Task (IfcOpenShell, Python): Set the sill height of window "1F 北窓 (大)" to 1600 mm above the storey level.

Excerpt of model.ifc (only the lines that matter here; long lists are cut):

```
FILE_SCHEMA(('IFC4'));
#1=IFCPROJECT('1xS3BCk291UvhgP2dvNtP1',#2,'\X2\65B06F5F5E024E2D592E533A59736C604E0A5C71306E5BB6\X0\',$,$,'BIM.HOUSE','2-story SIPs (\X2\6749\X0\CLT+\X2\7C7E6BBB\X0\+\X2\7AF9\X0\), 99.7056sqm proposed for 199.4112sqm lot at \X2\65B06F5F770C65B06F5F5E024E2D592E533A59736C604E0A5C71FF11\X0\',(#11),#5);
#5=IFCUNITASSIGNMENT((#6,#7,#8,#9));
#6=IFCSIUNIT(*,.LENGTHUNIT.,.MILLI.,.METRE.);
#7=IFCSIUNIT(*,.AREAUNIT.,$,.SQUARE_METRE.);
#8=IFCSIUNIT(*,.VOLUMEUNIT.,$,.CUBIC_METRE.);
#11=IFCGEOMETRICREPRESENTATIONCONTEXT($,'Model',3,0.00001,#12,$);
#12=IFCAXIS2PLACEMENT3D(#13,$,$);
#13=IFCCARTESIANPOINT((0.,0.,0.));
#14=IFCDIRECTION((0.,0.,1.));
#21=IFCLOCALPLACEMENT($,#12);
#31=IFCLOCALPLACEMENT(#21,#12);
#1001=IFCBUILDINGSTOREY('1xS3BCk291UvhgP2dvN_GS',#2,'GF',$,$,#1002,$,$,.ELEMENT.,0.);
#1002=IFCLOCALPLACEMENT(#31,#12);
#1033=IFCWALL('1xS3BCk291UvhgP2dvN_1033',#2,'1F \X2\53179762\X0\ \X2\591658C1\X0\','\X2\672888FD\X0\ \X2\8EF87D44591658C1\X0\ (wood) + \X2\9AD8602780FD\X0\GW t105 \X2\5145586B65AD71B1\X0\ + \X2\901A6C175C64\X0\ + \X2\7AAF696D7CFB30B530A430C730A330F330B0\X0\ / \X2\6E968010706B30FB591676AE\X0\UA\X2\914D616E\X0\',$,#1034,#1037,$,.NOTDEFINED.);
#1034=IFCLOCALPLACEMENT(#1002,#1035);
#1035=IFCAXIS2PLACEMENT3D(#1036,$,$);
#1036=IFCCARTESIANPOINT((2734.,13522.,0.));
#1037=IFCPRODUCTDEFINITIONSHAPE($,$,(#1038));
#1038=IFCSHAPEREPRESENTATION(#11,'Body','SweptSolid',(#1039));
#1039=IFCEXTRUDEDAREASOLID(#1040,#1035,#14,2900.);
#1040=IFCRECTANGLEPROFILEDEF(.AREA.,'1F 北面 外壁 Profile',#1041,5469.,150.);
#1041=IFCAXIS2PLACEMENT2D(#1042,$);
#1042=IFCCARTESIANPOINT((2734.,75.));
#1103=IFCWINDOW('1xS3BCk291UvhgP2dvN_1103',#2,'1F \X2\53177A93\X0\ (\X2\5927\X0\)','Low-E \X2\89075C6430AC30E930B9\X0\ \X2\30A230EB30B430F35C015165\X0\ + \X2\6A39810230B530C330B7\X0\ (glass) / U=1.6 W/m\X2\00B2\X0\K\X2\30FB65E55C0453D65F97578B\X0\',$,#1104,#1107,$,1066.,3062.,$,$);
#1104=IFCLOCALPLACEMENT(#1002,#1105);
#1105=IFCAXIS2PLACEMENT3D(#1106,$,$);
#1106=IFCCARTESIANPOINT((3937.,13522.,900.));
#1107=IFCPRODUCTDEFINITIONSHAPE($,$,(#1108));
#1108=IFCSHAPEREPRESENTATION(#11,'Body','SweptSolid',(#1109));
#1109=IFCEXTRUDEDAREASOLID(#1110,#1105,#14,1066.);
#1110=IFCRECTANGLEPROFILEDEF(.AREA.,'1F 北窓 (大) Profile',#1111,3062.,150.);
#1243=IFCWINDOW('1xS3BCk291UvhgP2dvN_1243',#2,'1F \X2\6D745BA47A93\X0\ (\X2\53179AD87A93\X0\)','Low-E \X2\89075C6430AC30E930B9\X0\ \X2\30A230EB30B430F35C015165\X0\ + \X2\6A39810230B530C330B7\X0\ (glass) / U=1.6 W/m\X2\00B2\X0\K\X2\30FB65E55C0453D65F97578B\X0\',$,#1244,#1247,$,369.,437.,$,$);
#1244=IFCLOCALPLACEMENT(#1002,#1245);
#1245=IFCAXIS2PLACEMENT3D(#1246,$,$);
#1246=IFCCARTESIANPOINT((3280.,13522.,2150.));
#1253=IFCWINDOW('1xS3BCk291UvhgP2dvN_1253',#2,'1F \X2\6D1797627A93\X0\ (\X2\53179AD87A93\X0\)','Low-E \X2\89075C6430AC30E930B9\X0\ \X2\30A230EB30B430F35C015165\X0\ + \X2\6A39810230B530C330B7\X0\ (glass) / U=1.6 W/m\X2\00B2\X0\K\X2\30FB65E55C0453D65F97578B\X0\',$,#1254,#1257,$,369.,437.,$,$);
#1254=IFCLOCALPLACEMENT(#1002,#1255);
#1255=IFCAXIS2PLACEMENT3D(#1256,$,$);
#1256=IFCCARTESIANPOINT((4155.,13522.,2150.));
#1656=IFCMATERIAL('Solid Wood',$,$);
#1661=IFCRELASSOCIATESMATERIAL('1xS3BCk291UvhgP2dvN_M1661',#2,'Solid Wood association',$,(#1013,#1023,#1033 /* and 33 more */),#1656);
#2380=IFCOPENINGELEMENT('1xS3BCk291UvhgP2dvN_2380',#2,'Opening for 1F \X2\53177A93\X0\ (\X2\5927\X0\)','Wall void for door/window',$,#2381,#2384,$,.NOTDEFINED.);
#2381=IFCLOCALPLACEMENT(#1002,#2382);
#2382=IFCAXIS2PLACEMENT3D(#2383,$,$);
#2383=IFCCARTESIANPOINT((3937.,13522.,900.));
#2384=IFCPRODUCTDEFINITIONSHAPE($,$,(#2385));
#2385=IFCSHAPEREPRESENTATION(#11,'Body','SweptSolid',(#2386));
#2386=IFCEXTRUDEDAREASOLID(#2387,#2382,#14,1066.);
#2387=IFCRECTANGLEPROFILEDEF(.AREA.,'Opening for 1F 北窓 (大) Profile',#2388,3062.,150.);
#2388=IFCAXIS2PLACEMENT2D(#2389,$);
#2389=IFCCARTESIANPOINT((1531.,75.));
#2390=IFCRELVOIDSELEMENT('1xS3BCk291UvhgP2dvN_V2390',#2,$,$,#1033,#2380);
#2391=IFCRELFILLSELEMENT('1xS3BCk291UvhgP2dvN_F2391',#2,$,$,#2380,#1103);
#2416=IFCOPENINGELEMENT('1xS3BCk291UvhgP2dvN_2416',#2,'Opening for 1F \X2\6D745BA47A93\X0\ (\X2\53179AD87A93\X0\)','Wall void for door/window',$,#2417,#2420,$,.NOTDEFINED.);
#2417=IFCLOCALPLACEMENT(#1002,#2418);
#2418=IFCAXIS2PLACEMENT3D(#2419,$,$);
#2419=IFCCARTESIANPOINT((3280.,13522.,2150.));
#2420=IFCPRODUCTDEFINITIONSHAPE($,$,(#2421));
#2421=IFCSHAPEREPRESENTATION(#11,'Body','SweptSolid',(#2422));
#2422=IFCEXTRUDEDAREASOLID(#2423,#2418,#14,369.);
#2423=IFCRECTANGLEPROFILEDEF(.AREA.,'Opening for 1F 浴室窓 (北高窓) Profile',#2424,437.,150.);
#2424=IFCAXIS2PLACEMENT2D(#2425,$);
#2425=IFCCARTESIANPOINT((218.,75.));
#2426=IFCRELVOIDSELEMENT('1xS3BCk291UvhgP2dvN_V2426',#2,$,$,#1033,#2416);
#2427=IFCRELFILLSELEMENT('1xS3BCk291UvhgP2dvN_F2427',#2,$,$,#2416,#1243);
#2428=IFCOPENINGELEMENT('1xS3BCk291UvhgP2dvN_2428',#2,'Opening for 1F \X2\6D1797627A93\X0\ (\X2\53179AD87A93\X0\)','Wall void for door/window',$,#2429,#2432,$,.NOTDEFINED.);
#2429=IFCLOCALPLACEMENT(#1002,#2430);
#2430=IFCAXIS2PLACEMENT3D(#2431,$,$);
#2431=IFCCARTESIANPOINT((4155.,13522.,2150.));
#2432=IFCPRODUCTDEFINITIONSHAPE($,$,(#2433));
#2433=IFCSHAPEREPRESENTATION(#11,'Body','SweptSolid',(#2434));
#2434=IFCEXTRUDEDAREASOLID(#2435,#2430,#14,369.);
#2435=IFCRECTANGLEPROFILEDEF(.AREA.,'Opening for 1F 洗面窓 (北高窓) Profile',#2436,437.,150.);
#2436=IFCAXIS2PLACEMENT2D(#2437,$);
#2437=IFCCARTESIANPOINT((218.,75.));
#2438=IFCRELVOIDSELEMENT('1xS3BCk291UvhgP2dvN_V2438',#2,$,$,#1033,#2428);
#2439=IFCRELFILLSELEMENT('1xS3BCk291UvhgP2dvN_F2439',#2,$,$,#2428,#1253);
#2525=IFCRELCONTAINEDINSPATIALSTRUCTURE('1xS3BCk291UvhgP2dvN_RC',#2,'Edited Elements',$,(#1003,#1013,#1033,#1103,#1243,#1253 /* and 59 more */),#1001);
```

```python
import numpy as np
import ifcopenshell
import ifcopenshell.api.geometry
import ifcopenshell.geom
import ifcopenshell.util.element
import ifcopenshell.util.placement
import ifcopenshell.util.shape
import ifcopenshell.util.unit

model = ifcopenshell.open("model.ifc")
unit_scale = ifcopenshell.util.unit.calculate_unit_scale(model)

window = model.by_id(1103)
opening = window.FillsVoids[0].RelatingOpeningElement
storey = ifcopenshell.util.element.get_container(window, ifc_class="IfcBuildingStorey")
level = ifcopenshell.util.placement.get_local_placement(storey.ObjectPlacement)[2, 3]

# The opening's origin need not be at the sill, so measure its lowest point.
shape = ifcopenshell.geom.create_shape(ifcopenshell.geom.settings(), opening)
bottom = ifcopenshell.util.shape.get_shape_bottom_elevation(shape, shape.geometry) / unit_scale
dz = level + 1600.0 - bottom

shift = np.array([0.0, 0.0, dz])
# The window is not placed relative to its opening, so move both.
for product in (opening, window):
    matrix = ifcopenshell.util.placement.get_local_placement(product.ObjectPlacement)
    matrix[:3, 3] += shift
    ifcopenshell.api.geometry.edit_object_placement(model, product=product, matrix=matrix, is_si=False)

print(f"moved by {dz * unit_scale:+.3f} m")

model.write("model_rev.ifc")
```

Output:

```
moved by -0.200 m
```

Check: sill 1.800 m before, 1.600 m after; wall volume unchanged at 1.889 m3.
